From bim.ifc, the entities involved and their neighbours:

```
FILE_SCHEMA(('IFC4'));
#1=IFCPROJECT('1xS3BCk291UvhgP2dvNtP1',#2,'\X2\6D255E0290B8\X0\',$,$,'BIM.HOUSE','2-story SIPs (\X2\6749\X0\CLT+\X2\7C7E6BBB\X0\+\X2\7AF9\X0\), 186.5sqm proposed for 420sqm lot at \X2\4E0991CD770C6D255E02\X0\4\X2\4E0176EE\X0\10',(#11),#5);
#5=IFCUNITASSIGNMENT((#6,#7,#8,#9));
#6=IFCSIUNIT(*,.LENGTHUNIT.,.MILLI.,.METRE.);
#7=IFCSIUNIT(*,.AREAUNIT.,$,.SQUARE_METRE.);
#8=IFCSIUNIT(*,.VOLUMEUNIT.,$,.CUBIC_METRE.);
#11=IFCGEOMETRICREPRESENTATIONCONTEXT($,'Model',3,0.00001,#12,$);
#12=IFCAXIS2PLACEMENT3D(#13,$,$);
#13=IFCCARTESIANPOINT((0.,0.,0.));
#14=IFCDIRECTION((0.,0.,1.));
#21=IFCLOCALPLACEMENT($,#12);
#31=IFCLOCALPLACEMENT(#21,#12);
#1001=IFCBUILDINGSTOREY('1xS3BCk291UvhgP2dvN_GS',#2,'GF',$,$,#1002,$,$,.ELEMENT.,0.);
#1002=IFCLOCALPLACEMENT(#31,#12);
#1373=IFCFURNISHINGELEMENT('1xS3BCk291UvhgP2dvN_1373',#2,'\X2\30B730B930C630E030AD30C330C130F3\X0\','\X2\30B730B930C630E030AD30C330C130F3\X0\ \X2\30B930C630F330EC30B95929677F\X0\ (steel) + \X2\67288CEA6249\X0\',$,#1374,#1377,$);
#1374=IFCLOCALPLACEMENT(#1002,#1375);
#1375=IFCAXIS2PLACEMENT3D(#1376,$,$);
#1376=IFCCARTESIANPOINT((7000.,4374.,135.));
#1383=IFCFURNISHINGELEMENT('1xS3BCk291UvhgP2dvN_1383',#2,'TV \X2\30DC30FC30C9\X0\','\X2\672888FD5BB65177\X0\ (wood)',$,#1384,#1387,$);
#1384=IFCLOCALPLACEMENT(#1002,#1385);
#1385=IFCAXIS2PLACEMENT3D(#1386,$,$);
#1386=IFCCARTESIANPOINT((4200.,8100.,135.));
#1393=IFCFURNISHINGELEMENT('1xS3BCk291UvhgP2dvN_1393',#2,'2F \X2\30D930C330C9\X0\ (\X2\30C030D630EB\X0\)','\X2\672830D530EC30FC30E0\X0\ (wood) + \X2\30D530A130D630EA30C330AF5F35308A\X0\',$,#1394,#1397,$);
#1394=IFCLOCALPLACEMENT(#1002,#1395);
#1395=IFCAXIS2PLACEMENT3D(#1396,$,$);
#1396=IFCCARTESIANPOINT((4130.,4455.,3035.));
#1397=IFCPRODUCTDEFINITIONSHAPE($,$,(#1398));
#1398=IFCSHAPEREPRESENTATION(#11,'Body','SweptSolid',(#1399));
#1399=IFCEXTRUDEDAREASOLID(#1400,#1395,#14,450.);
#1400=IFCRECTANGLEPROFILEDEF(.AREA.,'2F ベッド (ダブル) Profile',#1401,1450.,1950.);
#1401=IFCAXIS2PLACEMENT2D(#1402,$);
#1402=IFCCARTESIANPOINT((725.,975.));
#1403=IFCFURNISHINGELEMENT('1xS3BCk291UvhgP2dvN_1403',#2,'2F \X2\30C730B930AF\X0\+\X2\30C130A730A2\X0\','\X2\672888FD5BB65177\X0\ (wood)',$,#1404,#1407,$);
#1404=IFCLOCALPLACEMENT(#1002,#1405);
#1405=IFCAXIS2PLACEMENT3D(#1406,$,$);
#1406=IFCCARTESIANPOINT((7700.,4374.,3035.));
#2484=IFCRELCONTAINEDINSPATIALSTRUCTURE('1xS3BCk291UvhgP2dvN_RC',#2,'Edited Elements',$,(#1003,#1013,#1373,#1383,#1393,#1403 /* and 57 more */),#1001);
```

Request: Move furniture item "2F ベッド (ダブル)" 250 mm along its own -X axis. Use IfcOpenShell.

```python
import ifcopenshell
import ifcopenshell.api.geometry
import ifcopenshell.util.placement

model = ifcopenshell.open("bim.ifc")

item = model.by_guid("1xS3BCk291UvhgP2dvN_1393")
matrix = ifcopenshell.util.placement.get_local_placement(item.ObjectPlacement)
matrix[:3, 3] -= matrix[:3, 0] * 250.0
ifcopenshell.api.geometry.edit_object_placement(model, product=item, matrix=matrix, is_si=False)

print(ifcopenshell.util.placement.get_local_placement(item.ObjectPlacement).round(3) + 0.0)

model.write("bim_v2.ifc")
```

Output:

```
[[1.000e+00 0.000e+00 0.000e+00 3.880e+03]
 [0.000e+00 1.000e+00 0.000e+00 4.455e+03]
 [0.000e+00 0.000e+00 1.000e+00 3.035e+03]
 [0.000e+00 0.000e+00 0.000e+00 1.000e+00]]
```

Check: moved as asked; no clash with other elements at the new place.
